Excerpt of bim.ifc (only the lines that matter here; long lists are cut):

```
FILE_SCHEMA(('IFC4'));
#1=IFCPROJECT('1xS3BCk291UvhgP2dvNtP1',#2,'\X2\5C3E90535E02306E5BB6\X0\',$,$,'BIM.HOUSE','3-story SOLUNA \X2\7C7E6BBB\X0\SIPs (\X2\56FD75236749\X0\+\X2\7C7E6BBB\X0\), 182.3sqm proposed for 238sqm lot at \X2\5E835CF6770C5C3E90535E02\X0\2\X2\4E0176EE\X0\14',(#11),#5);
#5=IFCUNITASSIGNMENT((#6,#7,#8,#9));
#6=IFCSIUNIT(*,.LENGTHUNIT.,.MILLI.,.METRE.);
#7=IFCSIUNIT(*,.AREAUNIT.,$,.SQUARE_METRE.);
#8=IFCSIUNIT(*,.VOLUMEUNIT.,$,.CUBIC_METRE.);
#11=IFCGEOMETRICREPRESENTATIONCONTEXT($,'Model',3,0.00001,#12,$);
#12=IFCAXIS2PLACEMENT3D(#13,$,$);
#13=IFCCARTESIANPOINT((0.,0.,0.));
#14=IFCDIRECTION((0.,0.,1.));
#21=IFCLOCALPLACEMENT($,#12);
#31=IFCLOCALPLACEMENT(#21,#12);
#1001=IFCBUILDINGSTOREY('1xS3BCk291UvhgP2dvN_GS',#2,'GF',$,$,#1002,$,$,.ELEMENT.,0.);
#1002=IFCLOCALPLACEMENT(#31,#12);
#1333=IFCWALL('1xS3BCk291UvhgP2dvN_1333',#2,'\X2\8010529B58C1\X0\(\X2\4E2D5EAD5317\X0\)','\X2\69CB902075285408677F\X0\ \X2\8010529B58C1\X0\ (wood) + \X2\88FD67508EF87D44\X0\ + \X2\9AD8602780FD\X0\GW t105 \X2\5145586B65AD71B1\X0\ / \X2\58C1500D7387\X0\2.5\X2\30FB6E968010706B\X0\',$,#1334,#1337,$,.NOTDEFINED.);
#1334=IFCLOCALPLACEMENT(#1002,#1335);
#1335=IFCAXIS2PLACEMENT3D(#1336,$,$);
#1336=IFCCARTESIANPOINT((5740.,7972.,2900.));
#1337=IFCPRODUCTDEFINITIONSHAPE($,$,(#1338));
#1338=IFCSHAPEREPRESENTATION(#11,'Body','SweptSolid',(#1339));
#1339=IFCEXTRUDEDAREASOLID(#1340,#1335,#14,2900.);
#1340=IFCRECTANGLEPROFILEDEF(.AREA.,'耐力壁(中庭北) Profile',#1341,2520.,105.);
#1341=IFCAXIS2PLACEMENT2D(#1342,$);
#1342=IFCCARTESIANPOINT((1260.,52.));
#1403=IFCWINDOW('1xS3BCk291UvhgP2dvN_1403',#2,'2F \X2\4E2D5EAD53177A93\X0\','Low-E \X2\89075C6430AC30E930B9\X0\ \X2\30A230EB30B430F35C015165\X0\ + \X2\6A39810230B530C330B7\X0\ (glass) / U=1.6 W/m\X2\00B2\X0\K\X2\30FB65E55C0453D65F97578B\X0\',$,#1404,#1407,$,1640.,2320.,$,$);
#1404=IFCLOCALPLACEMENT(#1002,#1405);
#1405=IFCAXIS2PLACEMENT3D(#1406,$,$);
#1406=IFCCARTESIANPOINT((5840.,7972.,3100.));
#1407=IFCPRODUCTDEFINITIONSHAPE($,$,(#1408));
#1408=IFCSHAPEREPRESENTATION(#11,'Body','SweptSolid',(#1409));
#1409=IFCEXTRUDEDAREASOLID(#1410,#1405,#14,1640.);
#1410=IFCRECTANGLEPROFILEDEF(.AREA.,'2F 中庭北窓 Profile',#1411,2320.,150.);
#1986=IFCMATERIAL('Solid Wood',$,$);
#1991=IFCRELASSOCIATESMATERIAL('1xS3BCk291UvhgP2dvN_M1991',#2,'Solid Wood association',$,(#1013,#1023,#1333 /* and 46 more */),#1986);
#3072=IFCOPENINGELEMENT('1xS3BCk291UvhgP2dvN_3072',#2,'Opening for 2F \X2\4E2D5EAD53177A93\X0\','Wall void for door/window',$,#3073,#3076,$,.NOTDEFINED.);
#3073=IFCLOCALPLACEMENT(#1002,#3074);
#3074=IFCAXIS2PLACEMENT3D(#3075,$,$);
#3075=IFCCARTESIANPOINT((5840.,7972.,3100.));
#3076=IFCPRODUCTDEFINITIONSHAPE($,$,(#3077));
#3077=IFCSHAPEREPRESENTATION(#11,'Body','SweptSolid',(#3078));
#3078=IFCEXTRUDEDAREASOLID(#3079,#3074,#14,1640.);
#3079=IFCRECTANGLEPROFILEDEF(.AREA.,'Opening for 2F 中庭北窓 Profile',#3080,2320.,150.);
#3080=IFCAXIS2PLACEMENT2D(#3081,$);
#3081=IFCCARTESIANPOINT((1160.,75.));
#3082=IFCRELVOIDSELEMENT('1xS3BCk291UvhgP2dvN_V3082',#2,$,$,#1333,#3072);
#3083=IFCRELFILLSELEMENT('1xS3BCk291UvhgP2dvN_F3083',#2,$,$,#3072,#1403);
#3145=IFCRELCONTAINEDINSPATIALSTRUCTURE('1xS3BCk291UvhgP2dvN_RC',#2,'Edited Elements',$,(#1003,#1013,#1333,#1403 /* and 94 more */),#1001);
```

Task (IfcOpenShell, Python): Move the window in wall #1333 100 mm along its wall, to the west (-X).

```python
import ifcopenshell
import ifcopenshell.api.geometry
import ifcopenshell.util.placement

model = ifcopenshell.open("bim.ifc")

window = model.by_guid("1xS3BCk291UvhgP2dvN_1403")
opening = window.FillsVoids[0].RelatingOpeningElement
wall = opening.VoidsElements[0].RelatingBuildingElement

wall_matrix = ifcopenshell.util.placement.get_local_placement(wall.ObjectPlacement)
shift = wall_matrix[:3, 0] * -100.0
before = ifcopenshell.util.placement.get_local_placement(window.ObjectPlacement)[:3, 3].copy()

# The window is not placed relative to its opening, so move both.
for product in (opening, window):
    matrix = ifcopenshell.util.placement.get_local_placement(product.ObjectPlacement)
    matrix[:3, 3] += shift
    ifcopenshell.api.geometry.edit_object_placement(model, product=product, matrix=matrix, is_si=False)

after = ifcopenshell.util.placement.get_local_placement(window.ObjectPlacement)[:3, 3]
print("window moved by", (after - before).round(3) + 0.0)

model.write("bim-out.ifc")
```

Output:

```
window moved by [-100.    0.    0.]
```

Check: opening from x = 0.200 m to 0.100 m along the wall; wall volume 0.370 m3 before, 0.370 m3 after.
